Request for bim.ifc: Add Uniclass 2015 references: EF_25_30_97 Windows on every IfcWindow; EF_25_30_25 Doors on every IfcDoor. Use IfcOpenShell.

First a look at what the model holds.

```python
import ifcopenshell

model = ifcopenshell.open("bim.ifc")
print(model.schema)
print("classifications:", [c.Name for c in model.by_type("IfcClassification")])
for ifc_class in ("IfcDoor", "IfcRoof", "IfcStair", "IfcWall", "IfcWindow"):
    print(ifc_class, len(model.by_type(ifc_class)))
```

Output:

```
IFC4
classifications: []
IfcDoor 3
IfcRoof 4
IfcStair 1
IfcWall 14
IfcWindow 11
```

```python
import ifcopenshell
import ifcopenshell.api.classification

model = ifcopenshell.open("bim.ifc")

system = ifcopenshell.api.classification.add_classification(model, classification="Uniclass 2015")

codes = {
    "IfcWindow": ("EF_25_30_97", "Windows"),
    "IfcDoor": ("EF_25_30_25", "Doors"),
}
for ifc_class, (code, name) in codes.items():
    products = model.by_type(ifc_class)
    ifcopenshell.api.classification.add_reference(
        model, products=products, classification=system, identification=code, name=name
    )
    print(code, len(products))

model.write("bim_rev.ifc")
```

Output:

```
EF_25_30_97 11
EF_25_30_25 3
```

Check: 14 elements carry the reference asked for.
